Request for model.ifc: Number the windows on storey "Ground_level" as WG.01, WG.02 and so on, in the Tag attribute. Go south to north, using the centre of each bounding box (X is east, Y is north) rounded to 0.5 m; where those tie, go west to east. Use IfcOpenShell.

First a look at what the model holds.

```python
import ifcopenshell
import ifcopenshell.util.element
import ifcopenshell.util.placement

model = ifcopenshell.open("model.ifc")
print(model.schema)
storey = next(s for s in model.by_type("IfcBuildingStorey") if s.Name == "Ground_level")
windows = [e for e in ifcopenshell.util.element.get_decomposition(storey) if e.is_a("IfcWindow")]
for e in sorted(windows, key=lambda e: e.id()):
    origin = ifcopenshell.util.placement.get_local_placement(e.ObjectPlacement)[:3, 3]
    print(e.id(), e.Tag, e.Name, origin.round(2) + 0.0, sep=" | ")
```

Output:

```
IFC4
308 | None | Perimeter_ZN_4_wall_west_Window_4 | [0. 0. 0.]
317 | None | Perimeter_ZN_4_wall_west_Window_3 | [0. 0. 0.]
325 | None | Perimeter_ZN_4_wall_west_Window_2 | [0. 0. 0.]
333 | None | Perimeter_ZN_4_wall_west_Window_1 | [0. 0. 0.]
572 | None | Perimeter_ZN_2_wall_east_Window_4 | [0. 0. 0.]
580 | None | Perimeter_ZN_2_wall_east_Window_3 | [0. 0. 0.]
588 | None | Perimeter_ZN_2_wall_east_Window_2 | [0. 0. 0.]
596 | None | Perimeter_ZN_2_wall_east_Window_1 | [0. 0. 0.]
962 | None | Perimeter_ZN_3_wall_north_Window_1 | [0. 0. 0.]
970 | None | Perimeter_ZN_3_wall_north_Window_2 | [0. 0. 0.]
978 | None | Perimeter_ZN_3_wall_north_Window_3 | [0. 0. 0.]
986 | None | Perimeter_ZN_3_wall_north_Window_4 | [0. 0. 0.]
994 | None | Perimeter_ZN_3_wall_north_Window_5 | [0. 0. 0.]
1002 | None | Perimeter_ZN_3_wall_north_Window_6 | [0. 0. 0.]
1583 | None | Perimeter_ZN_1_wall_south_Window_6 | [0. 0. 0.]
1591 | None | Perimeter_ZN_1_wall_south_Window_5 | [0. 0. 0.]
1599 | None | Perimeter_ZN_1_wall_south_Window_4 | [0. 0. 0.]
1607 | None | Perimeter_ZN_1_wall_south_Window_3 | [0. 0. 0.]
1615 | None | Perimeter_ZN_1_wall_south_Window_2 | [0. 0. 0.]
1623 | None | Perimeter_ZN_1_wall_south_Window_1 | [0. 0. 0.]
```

```python
import ifcopenshell
import ifcopenshell.geom
import ifcopenshell.util.element
import ifcopenshell.util.shape

model = ifcopenshell.open("model.ifc")
settings = ifcopenshell.geom.settings()
settings.set("use-world-coords", True)


def centre(element):
    shape = ifcopenshell.geom.create_shape(settings, element)
    return ifcopenshell.util.shape.get_bbox_centroid(shape.geometry)


storey = next(s for s in model.by_type("IfcBuildingStorey") if s.Name == "Ground_level")
windows = [e for e in ifcopenshell.util.element.get_decomposition(storey) if e.is_a("IfcWindow")]

# Insertion points can sit at a corner or the storey origin, so sort by the geometry (in metres).
centres = {e: centre(e) for e in windows}
windows.sort(key=lambda e: (round(centres[e][1] / 0.5), centres[e][0]))

for i, e in enumerate(windows, start=1):
    number = f"WG.{i:02d}"
    e.Tag = number
    print(e.id(), number)

model.write("model_v2.ifc")
```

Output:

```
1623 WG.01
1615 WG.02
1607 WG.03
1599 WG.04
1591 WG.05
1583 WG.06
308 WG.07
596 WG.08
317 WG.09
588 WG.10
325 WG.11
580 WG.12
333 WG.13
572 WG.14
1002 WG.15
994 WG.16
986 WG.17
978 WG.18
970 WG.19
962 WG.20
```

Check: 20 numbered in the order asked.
